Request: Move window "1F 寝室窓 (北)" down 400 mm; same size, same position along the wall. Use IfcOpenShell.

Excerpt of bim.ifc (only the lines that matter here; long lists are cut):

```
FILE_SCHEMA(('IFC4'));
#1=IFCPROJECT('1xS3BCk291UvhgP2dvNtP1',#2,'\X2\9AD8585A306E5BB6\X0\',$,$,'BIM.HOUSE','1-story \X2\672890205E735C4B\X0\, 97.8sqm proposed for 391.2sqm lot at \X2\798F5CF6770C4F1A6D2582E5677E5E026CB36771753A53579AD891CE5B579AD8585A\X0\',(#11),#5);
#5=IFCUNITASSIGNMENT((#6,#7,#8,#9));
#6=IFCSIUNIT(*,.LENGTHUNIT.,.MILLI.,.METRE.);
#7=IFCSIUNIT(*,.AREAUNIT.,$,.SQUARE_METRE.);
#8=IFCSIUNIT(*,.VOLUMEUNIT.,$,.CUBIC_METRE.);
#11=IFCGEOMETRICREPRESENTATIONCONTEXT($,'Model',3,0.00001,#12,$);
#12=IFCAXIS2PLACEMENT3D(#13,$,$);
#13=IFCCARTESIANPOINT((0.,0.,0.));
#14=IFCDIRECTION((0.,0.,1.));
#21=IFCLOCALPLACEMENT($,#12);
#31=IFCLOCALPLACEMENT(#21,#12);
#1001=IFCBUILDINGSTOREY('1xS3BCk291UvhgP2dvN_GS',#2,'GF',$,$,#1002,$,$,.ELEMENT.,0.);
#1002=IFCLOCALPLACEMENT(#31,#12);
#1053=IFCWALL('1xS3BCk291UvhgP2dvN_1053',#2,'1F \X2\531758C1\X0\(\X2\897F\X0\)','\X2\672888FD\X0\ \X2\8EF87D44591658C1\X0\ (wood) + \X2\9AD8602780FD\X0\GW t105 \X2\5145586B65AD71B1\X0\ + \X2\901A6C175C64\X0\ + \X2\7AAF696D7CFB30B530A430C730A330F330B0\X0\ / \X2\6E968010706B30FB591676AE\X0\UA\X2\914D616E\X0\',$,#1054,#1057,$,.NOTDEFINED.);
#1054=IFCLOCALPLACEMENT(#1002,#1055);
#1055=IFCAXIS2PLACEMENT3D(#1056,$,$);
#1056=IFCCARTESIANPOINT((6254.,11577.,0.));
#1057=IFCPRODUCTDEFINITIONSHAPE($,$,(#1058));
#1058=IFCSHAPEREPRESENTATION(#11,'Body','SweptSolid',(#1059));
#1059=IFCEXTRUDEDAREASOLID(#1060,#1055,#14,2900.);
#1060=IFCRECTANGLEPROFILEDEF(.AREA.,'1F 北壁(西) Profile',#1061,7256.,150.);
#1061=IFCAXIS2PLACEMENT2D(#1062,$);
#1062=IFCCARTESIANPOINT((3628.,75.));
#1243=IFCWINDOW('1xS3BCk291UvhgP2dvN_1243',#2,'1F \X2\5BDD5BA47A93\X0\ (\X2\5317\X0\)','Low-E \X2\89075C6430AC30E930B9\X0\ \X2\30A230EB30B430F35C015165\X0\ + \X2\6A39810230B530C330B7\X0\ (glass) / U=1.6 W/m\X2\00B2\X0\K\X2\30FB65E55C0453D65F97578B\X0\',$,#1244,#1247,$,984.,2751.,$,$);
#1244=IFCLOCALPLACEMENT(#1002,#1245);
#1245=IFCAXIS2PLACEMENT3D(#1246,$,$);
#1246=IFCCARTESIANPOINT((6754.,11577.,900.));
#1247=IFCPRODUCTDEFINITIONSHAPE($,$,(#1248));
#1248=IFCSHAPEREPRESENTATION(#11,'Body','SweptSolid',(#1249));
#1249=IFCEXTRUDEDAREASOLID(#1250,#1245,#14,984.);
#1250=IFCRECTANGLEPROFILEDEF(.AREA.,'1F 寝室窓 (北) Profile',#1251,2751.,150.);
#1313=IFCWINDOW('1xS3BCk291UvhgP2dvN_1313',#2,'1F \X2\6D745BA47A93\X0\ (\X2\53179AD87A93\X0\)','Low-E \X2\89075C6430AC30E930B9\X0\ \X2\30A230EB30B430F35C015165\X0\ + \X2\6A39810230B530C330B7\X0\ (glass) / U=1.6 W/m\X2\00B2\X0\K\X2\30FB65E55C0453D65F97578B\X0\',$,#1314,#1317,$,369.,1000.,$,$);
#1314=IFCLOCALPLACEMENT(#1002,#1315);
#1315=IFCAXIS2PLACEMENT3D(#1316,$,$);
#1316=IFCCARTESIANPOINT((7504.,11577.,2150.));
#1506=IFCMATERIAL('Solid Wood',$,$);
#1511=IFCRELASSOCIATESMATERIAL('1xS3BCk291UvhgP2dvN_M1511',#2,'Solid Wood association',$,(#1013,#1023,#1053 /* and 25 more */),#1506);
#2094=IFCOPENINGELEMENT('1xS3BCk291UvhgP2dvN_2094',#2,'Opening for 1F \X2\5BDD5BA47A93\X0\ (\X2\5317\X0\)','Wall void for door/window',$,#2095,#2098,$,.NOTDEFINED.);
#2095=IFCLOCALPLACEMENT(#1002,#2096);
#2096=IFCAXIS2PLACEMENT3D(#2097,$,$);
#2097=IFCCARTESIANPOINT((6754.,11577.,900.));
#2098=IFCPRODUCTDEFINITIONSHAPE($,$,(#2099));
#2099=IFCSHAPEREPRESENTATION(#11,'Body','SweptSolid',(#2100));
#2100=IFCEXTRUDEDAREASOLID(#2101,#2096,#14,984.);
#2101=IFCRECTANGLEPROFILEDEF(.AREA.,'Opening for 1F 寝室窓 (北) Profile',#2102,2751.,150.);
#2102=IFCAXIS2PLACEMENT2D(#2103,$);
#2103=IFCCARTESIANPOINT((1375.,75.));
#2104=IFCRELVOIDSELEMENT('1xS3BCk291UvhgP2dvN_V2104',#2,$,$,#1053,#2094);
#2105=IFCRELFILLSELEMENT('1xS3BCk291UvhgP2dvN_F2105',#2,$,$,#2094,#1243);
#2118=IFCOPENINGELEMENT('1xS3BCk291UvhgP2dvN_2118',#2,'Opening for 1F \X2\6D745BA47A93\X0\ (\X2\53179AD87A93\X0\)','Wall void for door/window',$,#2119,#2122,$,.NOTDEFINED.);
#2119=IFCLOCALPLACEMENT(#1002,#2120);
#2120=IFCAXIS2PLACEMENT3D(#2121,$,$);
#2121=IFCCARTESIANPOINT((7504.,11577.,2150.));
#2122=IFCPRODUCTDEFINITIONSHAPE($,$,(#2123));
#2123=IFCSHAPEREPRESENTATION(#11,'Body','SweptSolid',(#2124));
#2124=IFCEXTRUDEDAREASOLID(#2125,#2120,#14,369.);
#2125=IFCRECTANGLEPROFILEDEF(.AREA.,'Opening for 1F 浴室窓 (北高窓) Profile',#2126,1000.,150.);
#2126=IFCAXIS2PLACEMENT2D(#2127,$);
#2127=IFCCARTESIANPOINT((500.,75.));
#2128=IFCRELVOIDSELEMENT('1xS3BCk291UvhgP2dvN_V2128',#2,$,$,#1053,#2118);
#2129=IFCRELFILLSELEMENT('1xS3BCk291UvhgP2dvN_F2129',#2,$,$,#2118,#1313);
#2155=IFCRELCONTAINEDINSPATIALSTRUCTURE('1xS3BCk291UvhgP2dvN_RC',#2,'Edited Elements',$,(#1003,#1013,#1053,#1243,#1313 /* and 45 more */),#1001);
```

```python
import numpy as np
import ifcopenshell
import ifcopenshell.api.geometry
import ifcopenshell.util.placement
import ifcopenshell.util.unit

model = ifcopenshell.open("bim.ifc")
unit_scale = ifcopenshell.util.unit.calculate_unit_scale(model)

window = model.by_guid("1xS3BCk291UvhgP2dvN_1243")
opening = window.FillsVoids[0].RelatingOpeningElement
dz = -400.0

shift = np.array([0.0, 0.0, dz])
# The window is not placed relative to its opening, so move both.
for product in (opening, window):
    matrix = ifcopenshell.util.placement.get_local_placement(product.ObjectPlacement)
    matrix[:3, 3] += shift
    ifcopenshell.api.geometry.edit_object_placement(model, product=product, matrix=matrix, is_si=False)

print(f"moved by {dz * unit_scale:+.3f} m")

model.write("bim_rev.ifc")
```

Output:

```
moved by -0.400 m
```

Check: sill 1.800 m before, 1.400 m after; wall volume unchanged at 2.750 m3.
